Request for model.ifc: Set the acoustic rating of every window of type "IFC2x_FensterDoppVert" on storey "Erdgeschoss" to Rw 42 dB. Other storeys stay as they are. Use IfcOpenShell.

First a look at what the model holds.

```python
import ifcopenshell
import ifcopenshell.util.element

model = ifcopenshell.open("model.ifc")
print(model.schema)
storey = next(s for s in model.by_type("IfcBuildingStorey") if s.Name == "Erdgeschoss")
windows = [e for e in ifcopenshell.util.element.get_decomposition(storey) if e.is_a("IfcWindow")]
seen = {}
for e in windows:
    element_type = ifcopenshell.util.element.get_type(e)
    key = (element_type.Name if element_type != e and element_type else None, ifcopenshell.util.element.get_pset(e, "Pset_WindowCommon", "AcousticRating"))
    seen[key] = seen.get(key, 0) + 1
for (name, value), count in sorted(seen.items(), key=str):
    print(count, "x", name, "|", value)
```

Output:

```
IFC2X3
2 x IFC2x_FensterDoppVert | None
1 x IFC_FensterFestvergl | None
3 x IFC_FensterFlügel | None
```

```python
import ifcopenshell
import ifcopenshell.api.pset
import ifcopenshell.util.element

model = ifcopenshell.open("model.ifc")

storey = next(s for s in model.by_type("IfcBuildingStorey") if s.Name == "Erdgeschoss")
windows = [e for e in ifcopenshell.util.element.get_decomposition(storey) if e.is_a("IfcWindow")]

count = 0
for e in windows:
    element_type = ifcopenshell.util.element.get_type(e)
    if element_type in (None, e) or element_type.Name != "IFC2x_FensterDoppVert":
        continue
    # add_pset returns the element's existing set when there is one.
    pset = ifcopenshell.api.pset.add_pset(model, product=e, name="Pset_WindowCommon")
    ifcopenshell.api.pset.edit_pset(model, pset=pset, properties={"AcousticRating": "Rw 42 dB"})
    count += 1

print(count, "windows updated")

model.write("model_updated.ifc")
```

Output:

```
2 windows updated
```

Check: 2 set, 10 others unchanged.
